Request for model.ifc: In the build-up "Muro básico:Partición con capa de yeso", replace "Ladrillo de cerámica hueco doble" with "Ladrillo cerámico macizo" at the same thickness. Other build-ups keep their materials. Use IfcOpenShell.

First a look at what the model holds.

```python
import ifcopenshell
import ifcopenshell.util.element

model = ifcopenshell.open("model.ifc")
print(model.schema)
for layer_set in model.by_type("IfcMaterialLayerSet"):
    if layer_set.LayerSetName == "Muro básico:Partición con capa de yeso":
        for layer in layer_set.MaterialLayers:
            print(layer.id(), layer.Material and layer.Material.Name, layer.LayerThickness, sep=" | ")
        print(len(ifcopenshell.util.element.get_elements_by_material(model, layer_set)), "elements and types use it")
print(sorted(m.Name for m in model.by_type("IfcMaterial") if m.Name)[:60])
```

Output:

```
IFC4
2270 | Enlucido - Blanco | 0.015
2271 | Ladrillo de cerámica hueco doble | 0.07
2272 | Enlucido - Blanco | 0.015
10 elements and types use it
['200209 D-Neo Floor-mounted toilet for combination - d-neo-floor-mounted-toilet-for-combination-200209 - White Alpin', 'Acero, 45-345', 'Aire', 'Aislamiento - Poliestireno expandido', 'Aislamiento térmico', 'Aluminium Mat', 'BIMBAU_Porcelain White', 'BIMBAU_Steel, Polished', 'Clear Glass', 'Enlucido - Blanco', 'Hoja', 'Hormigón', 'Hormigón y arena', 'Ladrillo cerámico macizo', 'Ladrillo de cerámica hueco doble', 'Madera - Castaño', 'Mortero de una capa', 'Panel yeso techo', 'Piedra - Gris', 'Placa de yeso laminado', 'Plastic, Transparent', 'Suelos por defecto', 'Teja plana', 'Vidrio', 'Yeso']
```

```python
import ifcopenshell
import ifcopenshell.api.material

model = ifcopenshell.open("model.ifc")

layer_set = next(s for s in model.by_type("IfcMaterialLayerSet") if s.LayerSetName == "Muro básico:Partición con capa de yeso")
layer = next(l for l in layer_set.MaterialLayers if l.Material and l.Material.Name == "Ladrillo de cerámica hueco doble")
material = next(m for m in model.by_type("IfcMaterial") if m.Name == "Ladrillo cerámico macizo")

# Point this one layer at the other material; renaming the old one would change it everywhere.
ifcopenshell.api.material.edit_layer(model, layer=layer, attributes={"Name": material.Name}, material=material)

print([l.Material.Name if l.Material else None for l in layer_set.MaterialLayers])

model.write("model_rev.ifc")
```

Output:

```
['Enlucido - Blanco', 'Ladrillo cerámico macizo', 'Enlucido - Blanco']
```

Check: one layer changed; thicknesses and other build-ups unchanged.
